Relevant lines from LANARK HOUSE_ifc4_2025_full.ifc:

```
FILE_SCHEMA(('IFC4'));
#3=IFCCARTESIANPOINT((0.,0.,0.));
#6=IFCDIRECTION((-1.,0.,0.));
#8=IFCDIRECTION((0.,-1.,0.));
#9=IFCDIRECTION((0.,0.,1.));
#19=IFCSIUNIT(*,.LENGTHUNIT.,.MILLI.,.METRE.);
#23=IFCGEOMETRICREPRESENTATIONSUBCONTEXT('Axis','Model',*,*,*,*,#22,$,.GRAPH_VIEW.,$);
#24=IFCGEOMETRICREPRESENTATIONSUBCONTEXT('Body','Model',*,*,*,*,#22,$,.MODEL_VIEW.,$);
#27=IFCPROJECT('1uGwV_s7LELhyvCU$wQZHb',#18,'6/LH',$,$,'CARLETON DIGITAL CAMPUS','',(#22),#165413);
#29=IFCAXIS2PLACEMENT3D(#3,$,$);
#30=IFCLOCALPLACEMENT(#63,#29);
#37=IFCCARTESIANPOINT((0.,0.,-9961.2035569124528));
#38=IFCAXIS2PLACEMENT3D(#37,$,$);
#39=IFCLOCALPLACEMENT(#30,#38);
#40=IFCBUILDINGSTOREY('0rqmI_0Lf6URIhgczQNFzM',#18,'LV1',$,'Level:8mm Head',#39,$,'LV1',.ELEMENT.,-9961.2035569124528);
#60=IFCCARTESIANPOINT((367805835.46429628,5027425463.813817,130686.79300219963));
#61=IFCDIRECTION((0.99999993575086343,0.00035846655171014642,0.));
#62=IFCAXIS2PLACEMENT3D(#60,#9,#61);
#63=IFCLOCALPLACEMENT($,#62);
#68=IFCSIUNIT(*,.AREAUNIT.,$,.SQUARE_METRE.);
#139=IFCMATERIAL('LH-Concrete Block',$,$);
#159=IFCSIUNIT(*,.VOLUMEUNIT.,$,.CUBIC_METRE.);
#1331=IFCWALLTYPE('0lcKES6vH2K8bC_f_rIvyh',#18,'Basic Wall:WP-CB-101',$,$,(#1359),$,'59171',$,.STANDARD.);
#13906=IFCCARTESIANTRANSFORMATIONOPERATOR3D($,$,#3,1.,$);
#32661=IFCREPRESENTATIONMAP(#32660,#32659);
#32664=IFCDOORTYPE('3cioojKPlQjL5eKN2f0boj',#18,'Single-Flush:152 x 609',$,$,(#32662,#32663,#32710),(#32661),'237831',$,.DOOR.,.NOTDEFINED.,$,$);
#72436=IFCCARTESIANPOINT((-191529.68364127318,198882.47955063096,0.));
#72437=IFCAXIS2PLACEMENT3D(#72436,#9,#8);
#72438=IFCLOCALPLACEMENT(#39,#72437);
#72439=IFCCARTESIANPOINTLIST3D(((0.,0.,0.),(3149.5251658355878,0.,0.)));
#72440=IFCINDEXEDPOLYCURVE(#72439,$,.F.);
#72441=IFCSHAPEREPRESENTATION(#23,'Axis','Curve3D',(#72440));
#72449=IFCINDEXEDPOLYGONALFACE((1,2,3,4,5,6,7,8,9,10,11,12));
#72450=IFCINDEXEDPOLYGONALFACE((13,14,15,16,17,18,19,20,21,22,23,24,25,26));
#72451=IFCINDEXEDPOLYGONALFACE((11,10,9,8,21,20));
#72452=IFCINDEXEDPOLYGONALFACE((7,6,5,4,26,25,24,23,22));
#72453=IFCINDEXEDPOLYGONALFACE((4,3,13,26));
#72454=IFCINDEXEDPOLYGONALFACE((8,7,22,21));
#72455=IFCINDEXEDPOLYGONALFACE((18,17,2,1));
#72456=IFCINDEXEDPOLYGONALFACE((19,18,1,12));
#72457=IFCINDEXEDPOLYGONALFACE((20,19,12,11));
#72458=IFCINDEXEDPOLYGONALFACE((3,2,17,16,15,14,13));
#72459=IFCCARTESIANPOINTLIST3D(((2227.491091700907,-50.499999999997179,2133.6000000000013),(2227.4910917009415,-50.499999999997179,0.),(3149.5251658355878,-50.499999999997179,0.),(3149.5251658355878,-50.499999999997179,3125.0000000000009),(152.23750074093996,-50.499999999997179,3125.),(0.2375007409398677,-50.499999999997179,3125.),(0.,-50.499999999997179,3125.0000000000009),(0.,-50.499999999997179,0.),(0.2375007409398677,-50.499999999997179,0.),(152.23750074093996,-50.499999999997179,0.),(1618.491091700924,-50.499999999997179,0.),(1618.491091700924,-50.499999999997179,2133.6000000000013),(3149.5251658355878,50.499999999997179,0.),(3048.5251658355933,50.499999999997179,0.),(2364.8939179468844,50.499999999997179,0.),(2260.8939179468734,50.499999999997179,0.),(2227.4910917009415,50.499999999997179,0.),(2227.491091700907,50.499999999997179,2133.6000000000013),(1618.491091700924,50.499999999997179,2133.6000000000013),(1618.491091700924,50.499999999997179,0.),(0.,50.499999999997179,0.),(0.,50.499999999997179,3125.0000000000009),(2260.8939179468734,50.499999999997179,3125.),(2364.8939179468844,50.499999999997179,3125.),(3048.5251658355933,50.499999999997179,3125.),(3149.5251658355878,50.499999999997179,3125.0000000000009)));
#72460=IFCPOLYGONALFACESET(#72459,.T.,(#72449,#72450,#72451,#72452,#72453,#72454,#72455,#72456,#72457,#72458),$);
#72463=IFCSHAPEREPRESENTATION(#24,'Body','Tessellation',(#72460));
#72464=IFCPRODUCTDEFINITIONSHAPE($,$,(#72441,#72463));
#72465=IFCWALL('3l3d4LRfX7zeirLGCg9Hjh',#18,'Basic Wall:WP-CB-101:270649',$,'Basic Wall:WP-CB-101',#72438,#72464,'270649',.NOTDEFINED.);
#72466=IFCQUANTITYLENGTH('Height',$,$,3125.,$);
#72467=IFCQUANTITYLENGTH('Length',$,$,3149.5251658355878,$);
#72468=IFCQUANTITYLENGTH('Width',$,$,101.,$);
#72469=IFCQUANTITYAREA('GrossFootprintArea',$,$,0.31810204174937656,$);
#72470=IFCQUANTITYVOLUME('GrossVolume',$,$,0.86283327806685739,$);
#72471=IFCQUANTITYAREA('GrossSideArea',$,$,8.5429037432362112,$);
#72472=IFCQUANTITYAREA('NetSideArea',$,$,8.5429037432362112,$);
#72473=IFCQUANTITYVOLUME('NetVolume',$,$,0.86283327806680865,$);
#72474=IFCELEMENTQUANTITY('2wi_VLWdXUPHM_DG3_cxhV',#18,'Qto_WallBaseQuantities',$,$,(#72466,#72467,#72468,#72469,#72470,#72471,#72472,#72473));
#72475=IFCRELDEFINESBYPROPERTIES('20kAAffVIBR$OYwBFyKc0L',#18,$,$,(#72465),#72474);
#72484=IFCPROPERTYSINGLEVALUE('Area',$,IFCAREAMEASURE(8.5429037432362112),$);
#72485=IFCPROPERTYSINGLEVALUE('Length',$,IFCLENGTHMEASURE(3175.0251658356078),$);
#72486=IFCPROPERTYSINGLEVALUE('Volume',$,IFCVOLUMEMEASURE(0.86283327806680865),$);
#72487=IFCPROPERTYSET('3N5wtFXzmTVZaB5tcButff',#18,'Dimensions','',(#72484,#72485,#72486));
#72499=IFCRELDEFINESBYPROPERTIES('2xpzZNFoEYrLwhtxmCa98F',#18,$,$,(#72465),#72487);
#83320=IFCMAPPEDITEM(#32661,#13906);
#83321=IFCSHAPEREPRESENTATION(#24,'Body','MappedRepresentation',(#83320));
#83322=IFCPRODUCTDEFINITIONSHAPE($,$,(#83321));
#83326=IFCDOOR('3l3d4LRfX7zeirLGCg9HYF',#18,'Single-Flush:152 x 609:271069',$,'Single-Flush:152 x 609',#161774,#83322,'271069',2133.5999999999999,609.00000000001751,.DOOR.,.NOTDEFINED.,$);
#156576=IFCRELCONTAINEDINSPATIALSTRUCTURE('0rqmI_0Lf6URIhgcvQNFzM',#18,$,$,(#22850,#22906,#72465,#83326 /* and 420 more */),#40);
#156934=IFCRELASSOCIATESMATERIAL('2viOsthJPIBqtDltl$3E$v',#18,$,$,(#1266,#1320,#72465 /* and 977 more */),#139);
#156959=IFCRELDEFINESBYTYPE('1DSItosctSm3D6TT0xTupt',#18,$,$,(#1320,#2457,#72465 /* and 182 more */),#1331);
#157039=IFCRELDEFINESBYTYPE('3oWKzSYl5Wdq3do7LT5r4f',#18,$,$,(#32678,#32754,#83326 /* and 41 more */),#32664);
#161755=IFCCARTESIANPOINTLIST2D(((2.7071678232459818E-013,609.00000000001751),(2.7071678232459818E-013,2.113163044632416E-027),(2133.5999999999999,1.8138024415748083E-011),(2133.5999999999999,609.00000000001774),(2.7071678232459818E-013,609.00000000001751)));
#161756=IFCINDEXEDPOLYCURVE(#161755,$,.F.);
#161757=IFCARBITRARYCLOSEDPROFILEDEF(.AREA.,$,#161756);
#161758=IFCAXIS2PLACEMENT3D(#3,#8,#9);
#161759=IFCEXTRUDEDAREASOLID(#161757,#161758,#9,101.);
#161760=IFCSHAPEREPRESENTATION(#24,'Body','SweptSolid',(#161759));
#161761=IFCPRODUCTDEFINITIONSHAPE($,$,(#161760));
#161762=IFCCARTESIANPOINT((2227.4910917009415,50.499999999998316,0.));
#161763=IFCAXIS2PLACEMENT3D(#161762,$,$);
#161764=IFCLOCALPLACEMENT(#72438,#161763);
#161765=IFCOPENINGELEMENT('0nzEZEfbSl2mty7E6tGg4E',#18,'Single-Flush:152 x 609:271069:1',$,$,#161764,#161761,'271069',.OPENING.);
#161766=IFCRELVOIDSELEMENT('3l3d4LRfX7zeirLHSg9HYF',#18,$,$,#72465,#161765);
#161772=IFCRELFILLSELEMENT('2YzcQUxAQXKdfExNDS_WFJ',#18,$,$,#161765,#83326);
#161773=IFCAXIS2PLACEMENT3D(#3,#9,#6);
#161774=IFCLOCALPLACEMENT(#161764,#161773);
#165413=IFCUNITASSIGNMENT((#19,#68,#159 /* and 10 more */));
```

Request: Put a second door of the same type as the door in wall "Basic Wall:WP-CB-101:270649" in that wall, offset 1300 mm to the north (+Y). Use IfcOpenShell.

```python
import ifcopenshell
import ifcopenshell.api.feature
import ifcopenshell.api.geometry
import ifcopenshell.api.pset
import ifcopenshell.api.root
import ifcopenshell.geom
import ifcopenshell.util.element
import ifcopenshell.util.placement
import ifcopenshell.util.shape
import ifcopenshell.util.unit

model = ifcopenshell.open("LANARK HOUSE_ifc4_2025_full.ifc")
unit_scale = ifcopenshell.util.unit.calculate_unit_scale(model)
area_scale = ifcopenshell.util.unit.calculate_unit_scale(model, "AREAUNIT")
volume_scale = ifcopenshell.util.unit.calculate_unit_scale(model, "VOLUMEUNIT")
settings = ifcopenshell.geom.settings()


def volume(element):
    """Net volume in cubic metres, openings subtracted."""
    shape = ifcopenshell.geom.create_shape(settings, element)
    return ifcopenshell.util.shape.get_volume(shape.geometry)


def reuse_history(source, copy):
    """copy_class also copies each property set's owner history, people and application; keep the originals."""
    for rel in copy.IsDefinedBy:
        if rel.is_a("IfcRelDefinesByProperties") and (history := rel.RelatingPropertyDefinition.OwnerHistory):
            rel.RelatingPropertyDefinition.OwnerHistory = source.OwnerHistory
            ifcopenshell.util.element.remove_deep2(model, history)


door = model.by_guid("3l3d4LRfX7zeirLGCg9HYF")
opening = door.FillsVoids[0].RelatingOpeningElement
wall = opening.VoidsElements[0].RelatingBuildingElement
before = volume(wall)
shift = ifcopenshell.util.placement.get_local_placement(wall.ObjectPlacement)[:3, 0] * -1.3 / unit_scale

# copy_class copies the void relationship, type, container and properties, but no geometry.
new_opening = ifcopenshell.api.root.copy_class(model, product=opening)
new_opening.Representation = ifcopenshell.util.element.copy_deep(
    model, opening.Representation, exclude=["IfcGeometricRepresentationContext", "IfcRepresentationMap"]
)
new_opening.Name = "Single-Flush:152 x 609"
new_opening.Tag = None
reuse_history(opening, new_opening)
new_door = ifcopenshell.api.root.copy_class(model, product=door)
new_door.Representation = ifcopenshell.util.element.copy_deep(
    model, door.Representation, exclude=["IfcGeometricRepresentationContext", "IfcRepresentationMap"]
)
new_door.Name = "Single-Flush:152 x 609"
new_door.Tag = None
reuse_history(door, new_door)
ifcopenshell.api.feature.add_filling(model, opening=new_opening, element=new_door)

for old, new in ((opening, new_opening), (door, new_door)):
    matrix = ifcopenshell.util.placement.get_local_placement(old.ObjectPlacement)
    matrix[:3, 3] += shift
    ifcopenshell.api.geometry.edit_object_placement(model, product=new, matrix=matrix, is_si=False)

after = volume(wall)
thickness = 0.101  # wall thickness in metres

# Update the wall's stored quantities.
qto = model.by_id(ifcopenshell.util.element.get_pset(wall, "Qto_WallBaseQuantities", should_inherit=False)["id"])
ifcopenshell.api.pset.edit_qto(model, qto=qto, properties={
    "NetSideArea": after / thickness / area_scale,
    "NetVolume": after / volume_scale,
})
pset = model.by_id(ifcopenshell.util.element.get_pset(wall, "Dimensions", should_inherit=False)["id"])
ifcopenshell.api.pset.edit_pset(model, pset=pset, properties={
    "Area": model.create_entity("IfcAreaMeasure", after / thickness / area_scale),
    "Volume": model.create_entity("IfcVolumeMeasure", after / volume_scale),
})

print(f"wall volume {before:.3f} -> {after:.3f} m3")

model.write("LANARK HOUSE_ifc4_2025_full_rev.ifc")
```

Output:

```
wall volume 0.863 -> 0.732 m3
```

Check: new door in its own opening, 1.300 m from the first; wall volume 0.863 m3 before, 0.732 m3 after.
